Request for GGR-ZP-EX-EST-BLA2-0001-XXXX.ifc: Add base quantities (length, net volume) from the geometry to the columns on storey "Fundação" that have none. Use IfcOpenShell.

First a look at what the model holds.

```python
import ifcopenshell
import ifcopenshell.util.element
import ifcopenshell.util.unit

model = ifcopenshell.open("GGR-ZP-EX-EST-BLA2-0001-XXXX.ifc")
print(model.schema)
for unit_type in ("LENGTHUNIT", "AREAUNIT", "VOLUMEUNIT"):
    print(unit_type, ifcopenshell.util.unit.calculate_unit_scale(model, unit_type))
storey = next(s for s in model.by_type("IfcBuildingStorey") if s.Name == "Fundação")
columns = [e for e in ifcopenshell.util.element.get_decomposition(storey) if e.is_a("IfcColumn")]
for e in sorted(columns, key=lambda e: e.id()):
    print(e.id(), e.is_a(), e.Name, list(ifcopenshell.util.element.get_psets(e, qtos_only=True)), sep=" | ")
```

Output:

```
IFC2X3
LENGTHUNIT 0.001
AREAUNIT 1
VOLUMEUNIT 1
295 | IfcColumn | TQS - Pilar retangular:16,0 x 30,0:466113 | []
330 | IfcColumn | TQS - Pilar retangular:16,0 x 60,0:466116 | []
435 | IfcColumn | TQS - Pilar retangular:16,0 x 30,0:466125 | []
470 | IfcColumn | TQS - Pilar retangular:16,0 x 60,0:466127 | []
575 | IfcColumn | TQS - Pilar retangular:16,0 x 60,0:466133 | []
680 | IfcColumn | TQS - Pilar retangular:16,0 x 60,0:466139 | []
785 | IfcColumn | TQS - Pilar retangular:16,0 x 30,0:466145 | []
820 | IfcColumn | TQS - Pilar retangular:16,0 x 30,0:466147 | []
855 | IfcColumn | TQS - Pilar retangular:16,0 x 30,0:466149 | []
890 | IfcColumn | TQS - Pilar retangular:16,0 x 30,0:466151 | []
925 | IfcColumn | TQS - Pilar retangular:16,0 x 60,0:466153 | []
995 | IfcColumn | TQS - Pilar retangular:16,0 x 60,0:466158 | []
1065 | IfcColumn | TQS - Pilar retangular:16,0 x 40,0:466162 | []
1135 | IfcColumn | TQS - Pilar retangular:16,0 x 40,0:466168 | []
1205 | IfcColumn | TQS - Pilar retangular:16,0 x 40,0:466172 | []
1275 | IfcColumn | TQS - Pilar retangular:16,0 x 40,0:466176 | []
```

```python
import ifcopenshell
import ifcopenshell.api.pset
import ifcopenshell.geom
import ifcopenshell.util.element
import ifcopenshell.util.shape
import ifcopenshell.util.unit

model = ifcopenshell.open("GGR-ZP-EX-EST-BLA2-0001-XXXX.ifc")
unit_scale = ifcopenshell.util.unit.calculate_unit_scale(model)
volume_scale = ifcopenshell.util.unit.calculate_unit_scale(model, "VOLUMEUNIT")
settings = ifcopenshell.geom.settings()

storey = next(s for s in model.by_type("IfcBuildingStorey") if s.Name == "Fundação")
columns = [e for e in ifcopenshell.util.element.get_decomposition(storey) if e.is_a("IfcColumn")]

for e in sorted(columns, key=lambda e: e.id()):
    if ifcopenshell.util.element.get_psets(e, qtos_only=True, should_inherit=False):
        continue
    # Geometry comes back in metres, in the element's own axes.
    shape = ifcopenshell.geom.create_shape(settings, e)
    values = {
        "Length": ifcopenshell.util.shape.get_z(shape.geometry) / unit_scale,
        "NetVolume": ifcopenshell.util.shape.get_volume(shape.geometry) / volume_scale,
    }
    qto = ifcopenshell.api.pset.add_qto(model, product=e, name="BaseQuantities")
    ifcopenshell.api.pset.edit_qto(model, qto=qto, properties=values)
    print(e.id(), {k: round(v, 3) for k, v in values.items()})

model.write("GGR-ZP-EX-EST-BLA2-0001-XXXX_edited.ifc")
```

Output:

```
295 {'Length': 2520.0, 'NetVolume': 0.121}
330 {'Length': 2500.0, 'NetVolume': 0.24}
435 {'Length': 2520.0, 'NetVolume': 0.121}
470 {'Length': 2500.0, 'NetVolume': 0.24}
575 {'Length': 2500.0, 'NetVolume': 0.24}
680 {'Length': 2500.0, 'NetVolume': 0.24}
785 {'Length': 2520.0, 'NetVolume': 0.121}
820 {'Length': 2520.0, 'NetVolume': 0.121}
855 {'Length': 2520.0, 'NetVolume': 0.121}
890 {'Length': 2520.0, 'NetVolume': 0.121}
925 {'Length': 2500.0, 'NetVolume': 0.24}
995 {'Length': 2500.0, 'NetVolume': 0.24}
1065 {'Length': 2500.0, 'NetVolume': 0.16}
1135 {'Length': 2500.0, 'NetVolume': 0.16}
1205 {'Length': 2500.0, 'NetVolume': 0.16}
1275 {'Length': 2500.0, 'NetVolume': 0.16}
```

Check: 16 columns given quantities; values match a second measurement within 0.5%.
